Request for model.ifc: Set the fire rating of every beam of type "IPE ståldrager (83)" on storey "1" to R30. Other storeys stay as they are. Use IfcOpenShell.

First a look at what the model holds.

```python
import ifcopenshell
import ifcopenshell.util.element

model = ifcopenshell.open("model.ifc")
print(model.schema)
storey = next(s for s in model.by_type("IfcBuildingStorey") if s.Name == "1")
beams = [e for e in ifcopenshell.util.element.get_decomposition(storey) if e.is_a("IfcBeam")]
seen = {}
for e in beams:
    element_type = ifcopenshell.util.element.get_type(e)
    key = (element_type.Name if element_type != e and element_type else None, ifcopenshell.util.element.get_pset(e, "Pset_BeamCommon", "FireRating"))
    seen[key] = seen.get(key, 0) + 1
for (name, value), count in sorted(seen.items(), key=str):
    print(count, "x", name, "|", value)
```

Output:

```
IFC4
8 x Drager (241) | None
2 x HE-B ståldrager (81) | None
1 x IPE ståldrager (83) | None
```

```python
import ifcopenshell
import ifcopenshell.api.pset
import ifcopenshell.util.element

model = ifcopenshell.open("model.ifc")

storey = next(s for s in model.by_type("IfcBuildingStorey") if s.Name == "1")
beams = [e for e in ifcopenshell.util.element.get_decomposition(storey) if e.is_a("IfcBeam")]

count = 0
for e in beams:
    element_type = ifcopenshell.util.element.get_type(e)
    if element_type in (None, e) or element_type.Name != "IPE ståldrager (83)":
        continue
    # add_pset returns the element's existing set when there is one.
    pset = ifcopenshell.api.pset.add_pset(model, product=e, name="Pset_BeamCommon")
    ifcopenshell.api.pset.edit_pset(model, pset=pset, properties={"FireRating": "R30"})
    count += 1

print(count, "beams updated")

model.write("model_v2.ifc")
```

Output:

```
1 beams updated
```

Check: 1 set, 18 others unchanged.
